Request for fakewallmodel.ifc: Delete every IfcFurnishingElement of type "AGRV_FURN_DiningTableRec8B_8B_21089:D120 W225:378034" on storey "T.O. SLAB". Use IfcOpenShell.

First a look at what the model holds.

```python
import ifcopenshell
import ifcopenshell.util.element

model = ifcopenshell.open("fakewallmodel.ifc")
print(model.schema)
storey = next(s for s in model.by_type("IfcBuildingStorey") if s.Name == "T.O. SLAB")
furniture = [e for e in ifcopenshell.util.element.get_decomposition(storey) if e.is_a("IfcFurnishingElement")]
seen = {}
for e in furniture:
    element_type = ifcopenshell.util.element.get_type(e)
    name = element_type.Name if element_type not in (None, e) else None
    seen[name] = seen.get(name, 0) + 1
for name, count in sorted(seen.items(), key=str):
    print(count, "x", name)
```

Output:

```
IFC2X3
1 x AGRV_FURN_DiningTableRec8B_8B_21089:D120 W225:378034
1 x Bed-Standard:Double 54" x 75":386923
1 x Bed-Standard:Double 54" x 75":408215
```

```python
import ifcopenshell
import ifcopenshell.api.root
import ifcopenshell.util.element

model = ifcopenshell.open("fakewallmodel.ifc")

storey = next(s for s in model.by_type("IfcBuildingStorey") if s.Name == "T.O. SLAB")
furniture = [e for e in ifcopenshell.util.element.get_decomposition(storey) if e.is_a("IfcFurnishingElement")]
targets = [e for e in furniture if (t := ifcopenshell.util.element.get_type(e)) not in (None, e) and t.Name == "AGRV_FURN_DiningTableRec8B_8B_21089:D120 W225:378034"]

for e in targets:
    ifcopenshell.api.root.remove_product(model, product=e)
print(len(targets), "removed")

model.write("fakewallmodel-out.ifc")
```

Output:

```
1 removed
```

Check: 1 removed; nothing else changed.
